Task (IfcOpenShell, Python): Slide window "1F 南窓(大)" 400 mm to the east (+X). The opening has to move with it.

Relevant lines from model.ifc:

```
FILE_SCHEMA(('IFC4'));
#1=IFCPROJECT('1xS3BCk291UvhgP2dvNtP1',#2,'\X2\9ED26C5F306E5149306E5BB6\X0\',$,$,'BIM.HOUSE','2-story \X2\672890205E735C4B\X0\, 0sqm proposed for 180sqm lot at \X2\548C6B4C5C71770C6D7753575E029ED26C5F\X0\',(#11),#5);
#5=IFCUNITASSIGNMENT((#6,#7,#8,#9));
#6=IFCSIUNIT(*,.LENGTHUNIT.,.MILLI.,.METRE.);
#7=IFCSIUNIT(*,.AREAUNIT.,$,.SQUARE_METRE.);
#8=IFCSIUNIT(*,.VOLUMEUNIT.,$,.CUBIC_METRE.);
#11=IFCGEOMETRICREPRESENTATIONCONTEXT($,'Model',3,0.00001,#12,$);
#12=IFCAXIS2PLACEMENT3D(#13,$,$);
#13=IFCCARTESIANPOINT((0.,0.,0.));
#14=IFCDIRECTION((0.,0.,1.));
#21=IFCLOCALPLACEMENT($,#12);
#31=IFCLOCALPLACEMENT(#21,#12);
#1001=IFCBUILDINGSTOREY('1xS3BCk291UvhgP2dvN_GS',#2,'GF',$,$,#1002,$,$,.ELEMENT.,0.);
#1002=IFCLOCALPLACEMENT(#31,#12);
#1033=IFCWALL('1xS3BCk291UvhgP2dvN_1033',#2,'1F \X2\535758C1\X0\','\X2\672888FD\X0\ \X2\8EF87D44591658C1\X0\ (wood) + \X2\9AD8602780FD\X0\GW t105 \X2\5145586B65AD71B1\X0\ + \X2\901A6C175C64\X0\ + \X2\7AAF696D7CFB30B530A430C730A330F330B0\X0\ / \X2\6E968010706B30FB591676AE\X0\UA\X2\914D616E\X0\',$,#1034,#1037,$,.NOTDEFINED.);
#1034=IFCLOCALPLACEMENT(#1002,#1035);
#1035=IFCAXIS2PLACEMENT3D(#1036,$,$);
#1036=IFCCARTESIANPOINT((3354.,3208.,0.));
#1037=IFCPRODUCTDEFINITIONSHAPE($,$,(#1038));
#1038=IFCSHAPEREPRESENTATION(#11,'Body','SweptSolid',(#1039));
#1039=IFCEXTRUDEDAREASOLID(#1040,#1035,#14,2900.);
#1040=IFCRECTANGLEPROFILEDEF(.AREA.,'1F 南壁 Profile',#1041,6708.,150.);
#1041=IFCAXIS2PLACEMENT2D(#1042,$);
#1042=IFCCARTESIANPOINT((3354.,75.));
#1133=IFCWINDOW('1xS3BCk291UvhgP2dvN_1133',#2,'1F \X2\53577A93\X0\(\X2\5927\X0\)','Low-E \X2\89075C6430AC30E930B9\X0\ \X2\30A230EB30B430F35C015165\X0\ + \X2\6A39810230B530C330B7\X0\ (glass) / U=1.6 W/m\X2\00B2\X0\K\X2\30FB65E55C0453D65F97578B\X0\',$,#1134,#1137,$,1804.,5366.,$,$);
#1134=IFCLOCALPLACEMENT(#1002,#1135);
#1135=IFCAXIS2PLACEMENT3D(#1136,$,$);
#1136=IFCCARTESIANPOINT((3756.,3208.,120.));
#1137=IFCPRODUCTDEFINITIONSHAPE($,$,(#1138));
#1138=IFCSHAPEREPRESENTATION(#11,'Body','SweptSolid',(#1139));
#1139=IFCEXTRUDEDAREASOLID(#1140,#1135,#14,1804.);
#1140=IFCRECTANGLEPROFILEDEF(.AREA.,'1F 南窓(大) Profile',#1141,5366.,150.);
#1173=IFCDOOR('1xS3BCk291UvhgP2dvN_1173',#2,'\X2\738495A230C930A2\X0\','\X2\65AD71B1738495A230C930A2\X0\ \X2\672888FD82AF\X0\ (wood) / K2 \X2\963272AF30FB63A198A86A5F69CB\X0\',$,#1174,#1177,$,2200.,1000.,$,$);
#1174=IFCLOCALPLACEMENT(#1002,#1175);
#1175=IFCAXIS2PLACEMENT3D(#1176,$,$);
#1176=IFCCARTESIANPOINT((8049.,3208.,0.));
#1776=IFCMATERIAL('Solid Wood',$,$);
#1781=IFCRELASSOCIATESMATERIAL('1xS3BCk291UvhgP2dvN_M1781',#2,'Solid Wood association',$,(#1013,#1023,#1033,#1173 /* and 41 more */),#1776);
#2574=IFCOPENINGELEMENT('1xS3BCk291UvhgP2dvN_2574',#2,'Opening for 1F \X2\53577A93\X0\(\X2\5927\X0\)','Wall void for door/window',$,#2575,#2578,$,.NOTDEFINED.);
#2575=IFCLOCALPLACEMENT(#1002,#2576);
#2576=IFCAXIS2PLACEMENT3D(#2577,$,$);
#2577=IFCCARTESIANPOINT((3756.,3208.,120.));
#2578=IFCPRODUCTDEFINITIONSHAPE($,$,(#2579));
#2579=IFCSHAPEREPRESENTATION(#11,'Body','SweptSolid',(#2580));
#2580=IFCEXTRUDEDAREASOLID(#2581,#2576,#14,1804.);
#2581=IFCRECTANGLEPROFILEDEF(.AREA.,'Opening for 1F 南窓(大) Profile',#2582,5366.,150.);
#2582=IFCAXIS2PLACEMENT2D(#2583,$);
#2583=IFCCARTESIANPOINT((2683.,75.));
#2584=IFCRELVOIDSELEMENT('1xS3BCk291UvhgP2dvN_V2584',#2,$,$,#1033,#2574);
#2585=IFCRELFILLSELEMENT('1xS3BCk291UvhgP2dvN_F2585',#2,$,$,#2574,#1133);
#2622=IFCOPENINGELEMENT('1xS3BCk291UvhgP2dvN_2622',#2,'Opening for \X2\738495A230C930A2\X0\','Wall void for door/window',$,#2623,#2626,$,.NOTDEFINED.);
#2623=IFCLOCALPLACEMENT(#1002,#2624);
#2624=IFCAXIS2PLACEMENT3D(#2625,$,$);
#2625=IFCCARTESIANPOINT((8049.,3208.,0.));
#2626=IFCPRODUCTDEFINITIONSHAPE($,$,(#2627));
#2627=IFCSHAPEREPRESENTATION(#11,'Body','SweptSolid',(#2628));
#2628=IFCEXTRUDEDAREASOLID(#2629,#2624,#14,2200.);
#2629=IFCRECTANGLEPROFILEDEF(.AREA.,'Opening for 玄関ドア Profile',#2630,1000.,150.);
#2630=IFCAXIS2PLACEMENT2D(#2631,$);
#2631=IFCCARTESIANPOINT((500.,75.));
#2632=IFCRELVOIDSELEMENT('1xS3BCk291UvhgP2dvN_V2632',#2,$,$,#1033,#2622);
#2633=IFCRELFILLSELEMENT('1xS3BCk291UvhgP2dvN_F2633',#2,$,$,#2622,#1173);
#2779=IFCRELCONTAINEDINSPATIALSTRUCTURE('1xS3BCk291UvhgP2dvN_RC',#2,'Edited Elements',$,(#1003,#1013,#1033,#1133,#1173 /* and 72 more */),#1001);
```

```python
import ifcopenshell
import ifcopenshell.api.geometry
import ifcopenshell.util.placement
import ifcopenshell.util.unit

model = ifcopenshell.open("model.ifc")
unit_scale = ifcopenshell.util.unit.calculate_unit_scale(model)

window = model.by_guid("1xS3BCk291UvhgP2dvN_1133")
opening = window.FillsVoids[0].RelatingOpeningElement
wall = opening.VoidsElements[0].RelatingBuildingElement

wall_matrix = ifcopenshell.util.placement.get_local_placement(wall.ObjectPlacement)
shift = wall_matrix[:3, 0] * 0.4 / unit_scale
before = ifcopenshell.util.placement.get_local_placement(window.ObjectPlacement)[:3, 3].copy()

# The window is not placed relative to its opening, so move both.
for product in (opening, window):
    matrix = ifcopenshell.util.placement.get_local_placement(product.ObjectPlacement)
    matrix[:3, 3] += shift
    ifcopenshell.api.geometry.edit_object_placement(model, product=product, matrix=matrix, is_si=False)

after = ifcopenshell.util.placement.get_local_placement(window.ObjectPlacement)[:3, 3]
print("window moved by", (after - before).round(3) + 0.0)

model.write("model_edited.ifc")
```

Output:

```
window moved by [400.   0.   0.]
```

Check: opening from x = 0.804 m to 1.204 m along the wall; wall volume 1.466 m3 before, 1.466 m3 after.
